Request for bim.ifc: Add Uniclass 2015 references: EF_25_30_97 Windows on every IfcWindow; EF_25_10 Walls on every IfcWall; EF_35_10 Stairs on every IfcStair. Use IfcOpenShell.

First a look at what the model holds.

```python
import ifcopenshell

model = ifcopenshell.open("bim.ifc")
print(model.schema)
print("classifications:", [c.Name for c in model.by_type("IfcClassification")])
for ifc_class in ("IfcDoor", "IfcRoof", "IfcStair", "IfcWall", "IfcWindow"):
    print(ifc_class, len(model.by_type(ifc_class)))
```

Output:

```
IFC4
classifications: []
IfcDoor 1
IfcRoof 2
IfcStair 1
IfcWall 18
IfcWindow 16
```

```python
import ifcopenshell
import ifcopenshell.api.classification

model = ifcopenshell.open("bim.ifc")

system = ifcopenshell.api.classification.add_classification(model, classification="Uniclass 2015")

codes = {
    "IfcWindow": ("EF_25_30_97", "Windows"),
    "IfcWall": ("EF_25_10", "Walls"),
    "IfcStair": ("EF_35_10", "Stairs"),
}
for ifc_class, (code, name) in codes.items():
    products = model.by_type(ifc_class)
    ifcopenshell.api.classification.add_reference(
        model, products=products, classification=system, identification=code, name=name
    )
    print(code, len(products))

model.write("bim_updated.ifc")
```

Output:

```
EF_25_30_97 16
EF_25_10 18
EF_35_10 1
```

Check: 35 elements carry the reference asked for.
